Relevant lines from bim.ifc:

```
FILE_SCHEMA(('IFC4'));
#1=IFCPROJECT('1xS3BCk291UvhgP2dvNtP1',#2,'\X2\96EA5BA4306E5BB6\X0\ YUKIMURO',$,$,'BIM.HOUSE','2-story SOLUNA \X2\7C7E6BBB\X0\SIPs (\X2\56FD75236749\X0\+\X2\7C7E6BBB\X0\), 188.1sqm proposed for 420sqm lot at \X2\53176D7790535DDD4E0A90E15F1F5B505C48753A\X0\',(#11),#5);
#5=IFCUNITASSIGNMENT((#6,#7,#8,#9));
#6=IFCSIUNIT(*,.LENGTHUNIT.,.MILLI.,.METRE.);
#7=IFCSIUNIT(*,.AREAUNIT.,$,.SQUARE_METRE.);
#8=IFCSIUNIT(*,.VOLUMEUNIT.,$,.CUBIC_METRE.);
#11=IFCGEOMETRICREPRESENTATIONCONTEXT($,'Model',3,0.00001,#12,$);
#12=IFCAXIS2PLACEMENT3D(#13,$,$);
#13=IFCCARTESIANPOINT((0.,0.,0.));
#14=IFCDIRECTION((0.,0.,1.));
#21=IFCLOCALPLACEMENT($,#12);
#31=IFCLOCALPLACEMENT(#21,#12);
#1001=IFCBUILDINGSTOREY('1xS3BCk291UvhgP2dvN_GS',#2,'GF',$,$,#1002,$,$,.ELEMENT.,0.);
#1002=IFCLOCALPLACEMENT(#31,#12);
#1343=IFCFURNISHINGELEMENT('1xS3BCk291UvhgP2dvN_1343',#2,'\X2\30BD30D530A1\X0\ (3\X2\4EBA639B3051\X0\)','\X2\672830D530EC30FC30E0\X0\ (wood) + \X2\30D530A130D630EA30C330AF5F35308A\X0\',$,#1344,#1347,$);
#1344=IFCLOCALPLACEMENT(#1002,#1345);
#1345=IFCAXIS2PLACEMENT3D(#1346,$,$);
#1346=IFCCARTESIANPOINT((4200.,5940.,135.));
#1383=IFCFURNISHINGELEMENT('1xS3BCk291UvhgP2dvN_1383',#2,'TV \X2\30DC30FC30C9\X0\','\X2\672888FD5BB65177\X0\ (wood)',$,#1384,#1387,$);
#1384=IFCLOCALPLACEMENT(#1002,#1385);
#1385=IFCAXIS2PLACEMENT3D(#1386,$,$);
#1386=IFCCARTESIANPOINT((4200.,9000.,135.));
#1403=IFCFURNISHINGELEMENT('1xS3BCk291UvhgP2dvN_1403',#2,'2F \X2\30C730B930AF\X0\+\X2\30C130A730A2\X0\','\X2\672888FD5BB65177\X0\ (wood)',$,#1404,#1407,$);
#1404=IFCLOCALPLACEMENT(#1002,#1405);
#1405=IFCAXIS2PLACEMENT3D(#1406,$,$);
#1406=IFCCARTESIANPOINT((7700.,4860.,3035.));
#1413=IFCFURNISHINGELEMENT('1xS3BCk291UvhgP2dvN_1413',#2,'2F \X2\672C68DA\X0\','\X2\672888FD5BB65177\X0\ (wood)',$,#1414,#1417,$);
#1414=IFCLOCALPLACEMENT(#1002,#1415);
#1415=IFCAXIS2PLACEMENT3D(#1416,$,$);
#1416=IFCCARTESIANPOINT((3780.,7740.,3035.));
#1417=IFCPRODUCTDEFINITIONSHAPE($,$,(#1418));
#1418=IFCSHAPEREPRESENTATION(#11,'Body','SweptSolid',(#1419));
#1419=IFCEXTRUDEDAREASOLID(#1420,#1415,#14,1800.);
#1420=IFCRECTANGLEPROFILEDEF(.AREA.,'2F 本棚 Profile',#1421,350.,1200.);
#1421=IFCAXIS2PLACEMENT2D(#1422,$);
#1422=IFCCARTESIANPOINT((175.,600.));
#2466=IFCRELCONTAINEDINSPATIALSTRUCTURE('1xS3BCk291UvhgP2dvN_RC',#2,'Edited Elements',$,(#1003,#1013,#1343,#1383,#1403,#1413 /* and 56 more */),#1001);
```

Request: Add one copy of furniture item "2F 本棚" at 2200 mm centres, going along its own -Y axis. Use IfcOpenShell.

```python
import ifcopenshell
import ifcopenshell.api.geometry
import ifcopenshell.api.root
import ifcopenshell.util.element
import ifcopenshell.util.placement

model = ifcopenshell.open("bim.ifc")


def reuse_history(source, copy):
    """copy_class also copies each property set's owner history, people and application; keep the originals."""
    for rel in copy.IsDefinedBy:
        if rel.is_a("IfcRelDefinesByProperties") and (history := rel.RelatingPropertyDefinition.OwnerHistory):
            rel.RelatingPropertyDefinition.OwnerHistory = source.OwnerHistory
            ifcopenshell.util.element.remove_deep2(model, history)


source = model.by_id(1413)
base = ifcopenshell.util.placement.get_local_placement(source.ObjectPlacement)
step = -base[:3, 1] * 2200.0

for i in range(1, 2):
    copy = ifcopenshell.api.root.copy_class(model, product=source)
    copy.Representation = ifcopenshell.util.element.copy_deep(
        model, source.Representation, exclude=["IfcGeometricRepresentationContext", "IfcRepresentationMap"]
    )
    reuse_history(source, copy)
    matrix = base.copy()
    matrix[:3, 3] += i * step
    print("added at", matrix[:3, 3].round(3) + 0.0)
    ifcopenshell.api.geometry.edit_object_placement(model, product=copy, matrix=matrix, is_si=False)

model.write("bim_updated.ifc")
```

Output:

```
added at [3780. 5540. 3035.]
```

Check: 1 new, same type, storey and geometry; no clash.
